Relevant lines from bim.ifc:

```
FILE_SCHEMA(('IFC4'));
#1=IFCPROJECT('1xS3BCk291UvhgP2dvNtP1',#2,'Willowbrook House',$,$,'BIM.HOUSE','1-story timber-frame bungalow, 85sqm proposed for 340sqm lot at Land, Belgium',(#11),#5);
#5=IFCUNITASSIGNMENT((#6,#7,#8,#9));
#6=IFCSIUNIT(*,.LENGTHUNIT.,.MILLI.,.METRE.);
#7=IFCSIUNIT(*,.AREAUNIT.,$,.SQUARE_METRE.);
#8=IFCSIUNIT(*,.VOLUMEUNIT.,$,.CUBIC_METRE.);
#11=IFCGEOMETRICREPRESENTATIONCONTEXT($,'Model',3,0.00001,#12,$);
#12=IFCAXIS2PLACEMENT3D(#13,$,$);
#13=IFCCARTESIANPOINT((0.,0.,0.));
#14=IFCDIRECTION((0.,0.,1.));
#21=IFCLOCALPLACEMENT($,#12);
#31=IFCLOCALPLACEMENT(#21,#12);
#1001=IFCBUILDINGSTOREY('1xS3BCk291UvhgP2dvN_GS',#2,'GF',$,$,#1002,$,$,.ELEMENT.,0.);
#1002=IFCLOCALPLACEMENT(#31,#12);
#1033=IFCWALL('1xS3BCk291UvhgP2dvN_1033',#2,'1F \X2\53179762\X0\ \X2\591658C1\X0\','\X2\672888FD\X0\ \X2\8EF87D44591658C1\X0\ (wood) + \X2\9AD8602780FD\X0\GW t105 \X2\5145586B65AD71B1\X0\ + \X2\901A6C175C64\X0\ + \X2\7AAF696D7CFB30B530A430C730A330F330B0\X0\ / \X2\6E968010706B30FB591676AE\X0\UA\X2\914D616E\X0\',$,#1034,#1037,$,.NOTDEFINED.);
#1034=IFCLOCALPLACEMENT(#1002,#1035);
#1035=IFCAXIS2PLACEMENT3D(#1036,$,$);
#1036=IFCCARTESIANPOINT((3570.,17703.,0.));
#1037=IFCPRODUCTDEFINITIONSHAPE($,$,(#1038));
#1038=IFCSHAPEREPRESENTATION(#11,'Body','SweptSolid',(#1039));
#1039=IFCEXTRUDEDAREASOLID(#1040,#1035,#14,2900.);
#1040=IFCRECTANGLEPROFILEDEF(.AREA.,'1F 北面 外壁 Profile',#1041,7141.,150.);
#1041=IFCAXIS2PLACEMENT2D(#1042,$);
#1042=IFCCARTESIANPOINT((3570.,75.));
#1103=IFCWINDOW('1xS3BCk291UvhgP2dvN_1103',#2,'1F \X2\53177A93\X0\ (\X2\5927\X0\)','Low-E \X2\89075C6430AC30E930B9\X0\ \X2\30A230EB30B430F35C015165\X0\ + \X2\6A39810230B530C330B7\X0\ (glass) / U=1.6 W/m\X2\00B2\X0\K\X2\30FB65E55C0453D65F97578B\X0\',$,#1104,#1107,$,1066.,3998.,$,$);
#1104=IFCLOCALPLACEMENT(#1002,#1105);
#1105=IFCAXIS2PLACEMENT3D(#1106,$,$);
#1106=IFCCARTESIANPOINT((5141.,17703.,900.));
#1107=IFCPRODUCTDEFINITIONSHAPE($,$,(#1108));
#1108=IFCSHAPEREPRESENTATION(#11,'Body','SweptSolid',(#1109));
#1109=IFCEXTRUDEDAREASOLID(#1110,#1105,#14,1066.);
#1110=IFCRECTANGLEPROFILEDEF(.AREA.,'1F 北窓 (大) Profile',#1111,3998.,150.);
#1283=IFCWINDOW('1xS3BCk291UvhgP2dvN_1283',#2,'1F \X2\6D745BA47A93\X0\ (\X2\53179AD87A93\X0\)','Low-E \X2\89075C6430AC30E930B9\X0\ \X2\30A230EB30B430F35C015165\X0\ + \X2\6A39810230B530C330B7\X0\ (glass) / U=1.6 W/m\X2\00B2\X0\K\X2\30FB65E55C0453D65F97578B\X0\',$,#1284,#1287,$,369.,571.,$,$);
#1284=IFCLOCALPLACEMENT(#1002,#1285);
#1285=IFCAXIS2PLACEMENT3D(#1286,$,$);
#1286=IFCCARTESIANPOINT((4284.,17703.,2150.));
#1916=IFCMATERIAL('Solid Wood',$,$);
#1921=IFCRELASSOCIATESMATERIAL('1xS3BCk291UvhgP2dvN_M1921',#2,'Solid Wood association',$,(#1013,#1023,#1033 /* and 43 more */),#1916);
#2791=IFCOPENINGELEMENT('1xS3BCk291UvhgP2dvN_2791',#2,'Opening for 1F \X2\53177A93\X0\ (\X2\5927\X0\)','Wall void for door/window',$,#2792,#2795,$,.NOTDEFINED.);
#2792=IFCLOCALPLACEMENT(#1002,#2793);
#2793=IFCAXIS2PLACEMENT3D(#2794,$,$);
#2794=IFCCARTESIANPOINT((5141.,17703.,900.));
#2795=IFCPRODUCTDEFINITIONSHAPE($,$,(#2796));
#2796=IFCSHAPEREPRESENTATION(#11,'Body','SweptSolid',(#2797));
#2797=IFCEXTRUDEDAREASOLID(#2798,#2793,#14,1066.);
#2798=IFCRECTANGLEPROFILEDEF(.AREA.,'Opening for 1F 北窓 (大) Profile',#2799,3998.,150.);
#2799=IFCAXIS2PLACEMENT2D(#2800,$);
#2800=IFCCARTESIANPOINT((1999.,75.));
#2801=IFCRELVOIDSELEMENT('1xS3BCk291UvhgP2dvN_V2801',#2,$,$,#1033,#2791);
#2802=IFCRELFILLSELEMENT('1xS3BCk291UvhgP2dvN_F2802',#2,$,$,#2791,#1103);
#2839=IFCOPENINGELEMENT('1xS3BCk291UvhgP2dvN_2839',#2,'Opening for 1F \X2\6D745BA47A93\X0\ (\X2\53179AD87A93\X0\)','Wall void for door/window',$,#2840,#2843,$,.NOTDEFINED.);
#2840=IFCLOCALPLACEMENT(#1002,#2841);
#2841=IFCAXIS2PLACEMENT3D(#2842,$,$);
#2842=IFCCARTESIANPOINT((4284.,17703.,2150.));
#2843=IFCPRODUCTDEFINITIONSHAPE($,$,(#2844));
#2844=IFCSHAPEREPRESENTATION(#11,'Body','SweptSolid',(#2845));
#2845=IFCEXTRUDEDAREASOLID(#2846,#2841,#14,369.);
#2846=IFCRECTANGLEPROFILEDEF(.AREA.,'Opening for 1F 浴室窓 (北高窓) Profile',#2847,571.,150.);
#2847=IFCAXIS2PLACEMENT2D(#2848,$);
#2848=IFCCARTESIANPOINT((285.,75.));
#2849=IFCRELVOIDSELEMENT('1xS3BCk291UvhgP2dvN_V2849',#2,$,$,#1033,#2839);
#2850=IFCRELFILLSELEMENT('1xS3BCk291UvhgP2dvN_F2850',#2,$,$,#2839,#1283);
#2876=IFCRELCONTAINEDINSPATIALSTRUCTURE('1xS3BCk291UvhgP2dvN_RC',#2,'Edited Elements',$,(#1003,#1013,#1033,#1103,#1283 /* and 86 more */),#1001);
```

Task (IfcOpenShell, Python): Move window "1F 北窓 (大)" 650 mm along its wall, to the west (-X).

```python
import ifcopenshell
import ifcopenshell.api.geometry
import ifcopenshell.util.placement

model = ifcopenshell.open("bim.ifc")

window = model.by_guid("1xS3BCk291UvhgP2dvN_1103")
opening = window.FillsVoids[0].RelatingOpeningElement
wall = opening.VoidsElements[0].RelatingBuildingElement

wall_matrix = ifcopenshell.util.placement.get_local_placement(wall.ObjectPlacement)
shift = wall_matrix[:3, 0] * -650.0
before = ifcopenshell.util.placement.get_local_placement(window.ObjectPlacement)[:3, 3].copy()

# The window is not placed relative to its opening, so move both.
for product in (opening, window):
    matrix = ifcopenshell.util.placement.get_local_placement(product.ObjectPlacement)
    matrix[:3, 3] += shift
    ifcopenshell.api.geometry.edit_object_placement(model, product=product, matrix=matrix, is_si=False)

after = ifcopenshell.util.placement.get_local_placement(window.ObjectPlacement)[:3, 3]
print("window moved by", (after - before).round(3) + 0.0)

model.write("bim-out.ifc")
```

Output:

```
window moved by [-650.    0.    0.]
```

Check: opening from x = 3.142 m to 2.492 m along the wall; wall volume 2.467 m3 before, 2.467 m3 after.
